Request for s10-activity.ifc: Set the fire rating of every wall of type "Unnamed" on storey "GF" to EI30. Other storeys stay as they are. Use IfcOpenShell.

First a look at what the model holds.

```python
import ifcopenshell
import ifcopenshell.util.element

model = ifcopenshell.open("s10-activity.ifc")
print(model.schema)
storey = next(s for s in model.by_type("IfcBuildingStorey") if s.Name == "GF")
walls = [e for e in ifcopenshell.util.element.get_decomposition(storey) if e.is_a("IfcWall")]
seen = {}
for e in walls:
    element_type = ifcopenshell.util.element.get_type(e)
    key = (element_type.Name if element_type != e and element_type else None, ifcopenshell.util.element.get_pset(e, "Pset_WallCommon", "FireRating"))
    seen[key] = seen.get(key, 0) + 1
for (name, value), count in sorted(seen.items(), key=str):
    print(count, "x", name, "|", value)
```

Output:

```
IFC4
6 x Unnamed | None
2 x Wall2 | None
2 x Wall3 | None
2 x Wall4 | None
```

```python
import ifcopenshell
import ifcopenshell.api.pset
import ifcopenshell.util.element

model = ifcopenshell.open("s10-activity.ifc")

storey = next(s for s in model.by_type("IfcBuildingStorey") if s.Name == "GF")
walls = [e for e in ifcopenshell.util.element.get_decomposition(storey) if e.is_a("IfcWall")]

count = 0
for e in walls:
    element_type = ifcopenshell.util.element.get_type(e)
    if element_type in (None, e) or element_type.Name != "Unnamed":
        continue
    # add_pset returns the element's existing set when there is one.
    pset = ifcopenshell.api.pset.add_pset(model, product=e, name="Pset_WallCommon")
    ifcopenshell.api.pset.edit_pset(model, pset=pset, properties={"FireRating": "EI30"})
    count += 1

print(count, "walls updated")

model.write("s10-activity_v2.ifc")
```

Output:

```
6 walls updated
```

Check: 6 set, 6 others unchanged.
